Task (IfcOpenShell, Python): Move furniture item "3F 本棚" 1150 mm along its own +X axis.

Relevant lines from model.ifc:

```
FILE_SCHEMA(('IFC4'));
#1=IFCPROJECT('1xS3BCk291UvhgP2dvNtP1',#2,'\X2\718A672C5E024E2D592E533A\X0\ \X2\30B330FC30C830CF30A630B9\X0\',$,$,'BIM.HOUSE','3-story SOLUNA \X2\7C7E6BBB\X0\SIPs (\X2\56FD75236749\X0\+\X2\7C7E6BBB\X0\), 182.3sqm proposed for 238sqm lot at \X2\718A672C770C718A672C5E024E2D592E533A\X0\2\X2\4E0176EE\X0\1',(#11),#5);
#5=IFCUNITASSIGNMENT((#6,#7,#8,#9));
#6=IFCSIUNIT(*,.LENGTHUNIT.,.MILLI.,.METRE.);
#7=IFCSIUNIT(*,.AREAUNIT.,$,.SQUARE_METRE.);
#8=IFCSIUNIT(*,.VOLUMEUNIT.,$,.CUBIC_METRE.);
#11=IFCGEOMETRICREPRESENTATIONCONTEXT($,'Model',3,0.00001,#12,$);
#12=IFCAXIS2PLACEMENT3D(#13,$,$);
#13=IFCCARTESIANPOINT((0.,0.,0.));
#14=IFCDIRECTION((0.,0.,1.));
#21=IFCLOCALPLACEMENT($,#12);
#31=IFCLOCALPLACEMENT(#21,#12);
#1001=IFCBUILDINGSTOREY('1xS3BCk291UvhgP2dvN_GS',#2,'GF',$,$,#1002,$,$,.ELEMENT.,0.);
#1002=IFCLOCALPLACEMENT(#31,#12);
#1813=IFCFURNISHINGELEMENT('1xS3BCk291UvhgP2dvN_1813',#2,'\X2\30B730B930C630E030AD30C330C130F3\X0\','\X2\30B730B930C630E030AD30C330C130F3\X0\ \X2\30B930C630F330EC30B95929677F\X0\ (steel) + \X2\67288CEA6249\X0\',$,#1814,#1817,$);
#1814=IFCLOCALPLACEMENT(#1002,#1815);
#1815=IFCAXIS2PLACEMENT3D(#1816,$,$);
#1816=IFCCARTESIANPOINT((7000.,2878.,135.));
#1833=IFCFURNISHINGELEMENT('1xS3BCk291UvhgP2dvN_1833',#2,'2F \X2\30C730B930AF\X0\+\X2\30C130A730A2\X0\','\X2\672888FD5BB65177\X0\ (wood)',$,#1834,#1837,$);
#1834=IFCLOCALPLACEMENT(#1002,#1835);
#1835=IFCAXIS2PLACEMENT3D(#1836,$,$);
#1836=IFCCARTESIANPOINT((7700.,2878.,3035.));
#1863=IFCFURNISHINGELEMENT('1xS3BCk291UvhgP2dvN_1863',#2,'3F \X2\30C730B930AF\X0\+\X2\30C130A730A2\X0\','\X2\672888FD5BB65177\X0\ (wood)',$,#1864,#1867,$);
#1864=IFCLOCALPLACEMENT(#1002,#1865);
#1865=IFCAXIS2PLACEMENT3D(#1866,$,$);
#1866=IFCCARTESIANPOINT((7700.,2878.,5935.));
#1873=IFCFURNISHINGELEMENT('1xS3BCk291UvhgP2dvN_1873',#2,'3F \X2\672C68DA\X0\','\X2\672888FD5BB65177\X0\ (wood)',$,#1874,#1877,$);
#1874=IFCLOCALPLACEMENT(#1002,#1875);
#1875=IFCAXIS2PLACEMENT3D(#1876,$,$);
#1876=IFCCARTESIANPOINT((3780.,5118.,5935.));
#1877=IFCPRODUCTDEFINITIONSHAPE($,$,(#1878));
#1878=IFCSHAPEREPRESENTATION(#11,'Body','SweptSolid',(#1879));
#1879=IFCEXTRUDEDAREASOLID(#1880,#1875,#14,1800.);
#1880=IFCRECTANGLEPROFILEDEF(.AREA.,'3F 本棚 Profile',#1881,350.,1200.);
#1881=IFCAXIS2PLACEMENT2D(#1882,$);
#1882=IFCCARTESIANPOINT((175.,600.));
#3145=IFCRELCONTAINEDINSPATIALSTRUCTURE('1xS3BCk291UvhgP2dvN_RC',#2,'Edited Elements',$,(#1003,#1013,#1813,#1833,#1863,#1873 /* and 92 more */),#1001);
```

```python
import ifcopenshell
import ifcopenshell.api.geometry
import ifcopenshell.util.placement
import ifcopenshell.util.unit

model = ifcopenshell.open("model.ifc")
unit_scale = ifcopenshell.util.unit.calculate_unit_scale(model)

item = model.by_guid("1xS3BCk291UvhgP2dvN_1873")
matrix = ifcopenshell.util.placement.get_local_placement(item.ObjectPlacement)
matrix[:3, 3] += matrix[:3, 0] * 1.15 / unit_scale
ifcopenshell.api.geometry.edit_object_placement(model, product=item, matrix=matrix, is_si=False)

print(ifcopenshell.util.placement.get_local_placement(item.ObjectPlacement).round(3) + 0.0)

model.write("model-out.ifc")
```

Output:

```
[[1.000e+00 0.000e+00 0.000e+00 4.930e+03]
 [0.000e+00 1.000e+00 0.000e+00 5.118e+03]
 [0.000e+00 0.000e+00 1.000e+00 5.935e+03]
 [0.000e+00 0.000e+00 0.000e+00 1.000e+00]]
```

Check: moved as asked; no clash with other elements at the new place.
